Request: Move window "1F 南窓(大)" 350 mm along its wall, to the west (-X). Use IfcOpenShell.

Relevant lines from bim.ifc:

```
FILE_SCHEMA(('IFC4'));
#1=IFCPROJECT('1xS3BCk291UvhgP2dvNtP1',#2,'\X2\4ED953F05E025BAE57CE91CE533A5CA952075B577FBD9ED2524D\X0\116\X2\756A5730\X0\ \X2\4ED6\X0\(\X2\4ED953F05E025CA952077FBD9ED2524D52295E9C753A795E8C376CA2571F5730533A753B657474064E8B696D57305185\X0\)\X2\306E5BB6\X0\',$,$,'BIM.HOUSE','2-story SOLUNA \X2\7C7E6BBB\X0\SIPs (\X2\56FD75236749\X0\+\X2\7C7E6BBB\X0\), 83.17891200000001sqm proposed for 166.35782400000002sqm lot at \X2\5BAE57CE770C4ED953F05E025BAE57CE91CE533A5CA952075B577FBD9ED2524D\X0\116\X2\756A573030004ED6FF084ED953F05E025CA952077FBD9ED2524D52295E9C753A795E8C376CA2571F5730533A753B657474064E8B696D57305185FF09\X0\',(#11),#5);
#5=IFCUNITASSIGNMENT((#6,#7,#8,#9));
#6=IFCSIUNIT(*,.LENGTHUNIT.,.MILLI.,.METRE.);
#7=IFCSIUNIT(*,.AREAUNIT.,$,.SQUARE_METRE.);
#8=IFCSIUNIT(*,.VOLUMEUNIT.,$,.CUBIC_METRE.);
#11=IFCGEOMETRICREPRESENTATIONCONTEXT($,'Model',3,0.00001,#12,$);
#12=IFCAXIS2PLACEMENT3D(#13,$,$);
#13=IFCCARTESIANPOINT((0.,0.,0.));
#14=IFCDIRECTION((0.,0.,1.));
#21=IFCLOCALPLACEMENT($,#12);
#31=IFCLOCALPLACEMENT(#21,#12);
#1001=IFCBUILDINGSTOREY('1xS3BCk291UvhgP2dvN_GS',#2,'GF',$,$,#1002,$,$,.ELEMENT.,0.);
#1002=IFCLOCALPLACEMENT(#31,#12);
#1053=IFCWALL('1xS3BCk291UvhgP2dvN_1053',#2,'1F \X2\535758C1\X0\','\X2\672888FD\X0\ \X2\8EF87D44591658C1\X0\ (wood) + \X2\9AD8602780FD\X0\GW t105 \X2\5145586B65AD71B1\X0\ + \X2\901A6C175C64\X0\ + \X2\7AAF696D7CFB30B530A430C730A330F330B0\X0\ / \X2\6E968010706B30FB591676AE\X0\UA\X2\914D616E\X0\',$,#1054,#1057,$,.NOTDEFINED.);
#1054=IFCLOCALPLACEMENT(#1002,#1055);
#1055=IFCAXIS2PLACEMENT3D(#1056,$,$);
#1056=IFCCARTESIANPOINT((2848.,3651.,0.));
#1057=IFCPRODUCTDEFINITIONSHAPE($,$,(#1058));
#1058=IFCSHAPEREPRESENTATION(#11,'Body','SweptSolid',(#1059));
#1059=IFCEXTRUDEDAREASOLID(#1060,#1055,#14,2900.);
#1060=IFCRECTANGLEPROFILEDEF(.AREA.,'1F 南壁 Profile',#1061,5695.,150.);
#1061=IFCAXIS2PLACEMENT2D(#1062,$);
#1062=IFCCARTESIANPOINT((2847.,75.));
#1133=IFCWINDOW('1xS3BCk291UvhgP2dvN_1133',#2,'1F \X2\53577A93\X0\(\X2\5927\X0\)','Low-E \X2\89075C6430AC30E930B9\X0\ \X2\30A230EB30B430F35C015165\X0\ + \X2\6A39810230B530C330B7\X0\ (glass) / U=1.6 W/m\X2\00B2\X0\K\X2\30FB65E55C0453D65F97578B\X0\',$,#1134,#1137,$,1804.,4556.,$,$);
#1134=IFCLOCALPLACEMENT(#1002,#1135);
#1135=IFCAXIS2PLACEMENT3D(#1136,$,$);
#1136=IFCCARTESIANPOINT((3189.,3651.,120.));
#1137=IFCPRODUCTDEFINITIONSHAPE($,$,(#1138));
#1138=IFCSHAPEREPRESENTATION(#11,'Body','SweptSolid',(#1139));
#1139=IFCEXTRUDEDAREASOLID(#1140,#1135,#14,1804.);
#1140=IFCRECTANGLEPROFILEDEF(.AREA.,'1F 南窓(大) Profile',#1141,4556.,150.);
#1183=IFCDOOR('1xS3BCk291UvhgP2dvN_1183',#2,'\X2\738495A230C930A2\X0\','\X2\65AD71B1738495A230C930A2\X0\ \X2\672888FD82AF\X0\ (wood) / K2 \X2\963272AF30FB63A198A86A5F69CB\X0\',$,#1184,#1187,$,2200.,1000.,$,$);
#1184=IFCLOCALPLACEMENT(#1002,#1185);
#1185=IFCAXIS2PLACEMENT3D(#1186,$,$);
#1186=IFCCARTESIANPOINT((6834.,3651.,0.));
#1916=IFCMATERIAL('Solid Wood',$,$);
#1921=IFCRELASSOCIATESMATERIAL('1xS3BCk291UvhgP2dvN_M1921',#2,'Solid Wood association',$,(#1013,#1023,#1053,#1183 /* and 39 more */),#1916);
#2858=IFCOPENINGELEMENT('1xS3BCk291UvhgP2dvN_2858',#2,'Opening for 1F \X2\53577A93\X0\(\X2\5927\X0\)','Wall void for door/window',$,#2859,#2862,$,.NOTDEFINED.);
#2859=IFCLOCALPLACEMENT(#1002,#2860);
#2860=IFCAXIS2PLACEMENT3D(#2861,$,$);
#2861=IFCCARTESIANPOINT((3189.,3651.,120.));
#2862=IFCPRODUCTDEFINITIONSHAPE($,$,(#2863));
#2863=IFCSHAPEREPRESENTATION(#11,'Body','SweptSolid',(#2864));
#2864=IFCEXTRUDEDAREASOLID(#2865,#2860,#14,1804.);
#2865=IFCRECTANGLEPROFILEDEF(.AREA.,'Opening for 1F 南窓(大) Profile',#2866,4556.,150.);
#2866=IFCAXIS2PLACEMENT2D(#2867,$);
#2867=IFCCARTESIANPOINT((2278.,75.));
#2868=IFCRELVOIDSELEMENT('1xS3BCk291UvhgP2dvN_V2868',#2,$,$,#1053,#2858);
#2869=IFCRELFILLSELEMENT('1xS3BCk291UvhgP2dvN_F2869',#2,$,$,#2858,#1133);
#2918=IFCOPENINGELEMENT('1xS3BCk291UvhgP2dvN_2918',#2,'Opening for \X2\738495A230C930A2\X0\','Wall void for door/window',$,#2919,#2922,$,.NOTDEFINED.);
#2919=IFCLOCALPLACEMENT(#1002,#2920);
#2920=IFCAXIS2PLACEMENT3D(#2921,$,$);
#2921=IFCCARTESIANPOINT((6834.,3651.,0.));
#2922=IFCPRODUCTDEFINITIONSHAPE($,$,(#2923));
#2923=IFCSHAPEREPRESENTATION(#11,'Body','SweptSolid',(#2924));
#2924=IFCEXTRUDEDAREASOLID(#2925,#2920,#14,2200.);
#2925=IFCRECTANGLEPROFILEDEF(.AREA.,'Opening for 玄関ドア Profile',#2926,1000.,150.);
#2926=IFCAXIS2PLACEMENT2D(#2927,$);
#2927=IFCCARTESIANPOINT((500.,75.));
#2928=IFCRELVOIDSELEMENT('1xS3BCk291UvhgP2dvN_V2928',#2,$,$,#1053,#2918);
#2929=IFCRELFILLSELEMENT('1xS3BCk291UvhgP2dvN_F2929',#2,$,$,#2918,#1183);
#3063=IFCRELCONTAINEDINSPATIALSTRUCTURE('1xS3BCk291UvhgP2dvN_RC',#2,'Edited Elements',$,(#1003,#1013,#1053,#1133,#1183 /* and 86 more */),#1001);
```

```python
import ifcopenshell
import ifcopenshell.api.geometry
import ifcopenshell.util.placement
import ifcopenshell.util.unit

model = ifcopenshell.open("bim.ifc")
unit_scale = ifcopenshell.util.unit.calculate_unit_scale(model)

window = model.by_id(1133)
opening = window.FillsVoids[0].RelatingOpeningElement
wall = opening.VoidsElements[0].RelatingBuildingElement

wall_matrix = ifcopenshell.util.placement.get_local_placement(wall.ObjectPlacement)
shift = wall_matrix[:3, 0] * -0.35 / unit_scale
before = ifcopenshell.util.placement.get_local_placement(window.ObjectPlacement)[:3, 3].copy()

# The window is not placed relative to its opening, so move both.
for product in (opening, window):
    matrix = ifcopenshell.util.placement.get_local_placement(product.ObjectPlacement)
    matrix[:3, 3] += shift
    ifcopenshell.api.geometry.edit_object_placement(model, product=product, matrix=matrix, is_si=False)

after = ifcopenshell.util.placement.get_local_placement(window.ObjectPlacement)[:3, 3]
print("window moved by", (after - before).round(3) + 0.0)

model.write("bim-out.ifc")
```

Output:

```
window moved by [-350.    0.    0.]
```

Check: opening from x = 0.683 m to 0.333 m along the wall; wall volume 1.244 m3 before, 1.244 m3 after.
